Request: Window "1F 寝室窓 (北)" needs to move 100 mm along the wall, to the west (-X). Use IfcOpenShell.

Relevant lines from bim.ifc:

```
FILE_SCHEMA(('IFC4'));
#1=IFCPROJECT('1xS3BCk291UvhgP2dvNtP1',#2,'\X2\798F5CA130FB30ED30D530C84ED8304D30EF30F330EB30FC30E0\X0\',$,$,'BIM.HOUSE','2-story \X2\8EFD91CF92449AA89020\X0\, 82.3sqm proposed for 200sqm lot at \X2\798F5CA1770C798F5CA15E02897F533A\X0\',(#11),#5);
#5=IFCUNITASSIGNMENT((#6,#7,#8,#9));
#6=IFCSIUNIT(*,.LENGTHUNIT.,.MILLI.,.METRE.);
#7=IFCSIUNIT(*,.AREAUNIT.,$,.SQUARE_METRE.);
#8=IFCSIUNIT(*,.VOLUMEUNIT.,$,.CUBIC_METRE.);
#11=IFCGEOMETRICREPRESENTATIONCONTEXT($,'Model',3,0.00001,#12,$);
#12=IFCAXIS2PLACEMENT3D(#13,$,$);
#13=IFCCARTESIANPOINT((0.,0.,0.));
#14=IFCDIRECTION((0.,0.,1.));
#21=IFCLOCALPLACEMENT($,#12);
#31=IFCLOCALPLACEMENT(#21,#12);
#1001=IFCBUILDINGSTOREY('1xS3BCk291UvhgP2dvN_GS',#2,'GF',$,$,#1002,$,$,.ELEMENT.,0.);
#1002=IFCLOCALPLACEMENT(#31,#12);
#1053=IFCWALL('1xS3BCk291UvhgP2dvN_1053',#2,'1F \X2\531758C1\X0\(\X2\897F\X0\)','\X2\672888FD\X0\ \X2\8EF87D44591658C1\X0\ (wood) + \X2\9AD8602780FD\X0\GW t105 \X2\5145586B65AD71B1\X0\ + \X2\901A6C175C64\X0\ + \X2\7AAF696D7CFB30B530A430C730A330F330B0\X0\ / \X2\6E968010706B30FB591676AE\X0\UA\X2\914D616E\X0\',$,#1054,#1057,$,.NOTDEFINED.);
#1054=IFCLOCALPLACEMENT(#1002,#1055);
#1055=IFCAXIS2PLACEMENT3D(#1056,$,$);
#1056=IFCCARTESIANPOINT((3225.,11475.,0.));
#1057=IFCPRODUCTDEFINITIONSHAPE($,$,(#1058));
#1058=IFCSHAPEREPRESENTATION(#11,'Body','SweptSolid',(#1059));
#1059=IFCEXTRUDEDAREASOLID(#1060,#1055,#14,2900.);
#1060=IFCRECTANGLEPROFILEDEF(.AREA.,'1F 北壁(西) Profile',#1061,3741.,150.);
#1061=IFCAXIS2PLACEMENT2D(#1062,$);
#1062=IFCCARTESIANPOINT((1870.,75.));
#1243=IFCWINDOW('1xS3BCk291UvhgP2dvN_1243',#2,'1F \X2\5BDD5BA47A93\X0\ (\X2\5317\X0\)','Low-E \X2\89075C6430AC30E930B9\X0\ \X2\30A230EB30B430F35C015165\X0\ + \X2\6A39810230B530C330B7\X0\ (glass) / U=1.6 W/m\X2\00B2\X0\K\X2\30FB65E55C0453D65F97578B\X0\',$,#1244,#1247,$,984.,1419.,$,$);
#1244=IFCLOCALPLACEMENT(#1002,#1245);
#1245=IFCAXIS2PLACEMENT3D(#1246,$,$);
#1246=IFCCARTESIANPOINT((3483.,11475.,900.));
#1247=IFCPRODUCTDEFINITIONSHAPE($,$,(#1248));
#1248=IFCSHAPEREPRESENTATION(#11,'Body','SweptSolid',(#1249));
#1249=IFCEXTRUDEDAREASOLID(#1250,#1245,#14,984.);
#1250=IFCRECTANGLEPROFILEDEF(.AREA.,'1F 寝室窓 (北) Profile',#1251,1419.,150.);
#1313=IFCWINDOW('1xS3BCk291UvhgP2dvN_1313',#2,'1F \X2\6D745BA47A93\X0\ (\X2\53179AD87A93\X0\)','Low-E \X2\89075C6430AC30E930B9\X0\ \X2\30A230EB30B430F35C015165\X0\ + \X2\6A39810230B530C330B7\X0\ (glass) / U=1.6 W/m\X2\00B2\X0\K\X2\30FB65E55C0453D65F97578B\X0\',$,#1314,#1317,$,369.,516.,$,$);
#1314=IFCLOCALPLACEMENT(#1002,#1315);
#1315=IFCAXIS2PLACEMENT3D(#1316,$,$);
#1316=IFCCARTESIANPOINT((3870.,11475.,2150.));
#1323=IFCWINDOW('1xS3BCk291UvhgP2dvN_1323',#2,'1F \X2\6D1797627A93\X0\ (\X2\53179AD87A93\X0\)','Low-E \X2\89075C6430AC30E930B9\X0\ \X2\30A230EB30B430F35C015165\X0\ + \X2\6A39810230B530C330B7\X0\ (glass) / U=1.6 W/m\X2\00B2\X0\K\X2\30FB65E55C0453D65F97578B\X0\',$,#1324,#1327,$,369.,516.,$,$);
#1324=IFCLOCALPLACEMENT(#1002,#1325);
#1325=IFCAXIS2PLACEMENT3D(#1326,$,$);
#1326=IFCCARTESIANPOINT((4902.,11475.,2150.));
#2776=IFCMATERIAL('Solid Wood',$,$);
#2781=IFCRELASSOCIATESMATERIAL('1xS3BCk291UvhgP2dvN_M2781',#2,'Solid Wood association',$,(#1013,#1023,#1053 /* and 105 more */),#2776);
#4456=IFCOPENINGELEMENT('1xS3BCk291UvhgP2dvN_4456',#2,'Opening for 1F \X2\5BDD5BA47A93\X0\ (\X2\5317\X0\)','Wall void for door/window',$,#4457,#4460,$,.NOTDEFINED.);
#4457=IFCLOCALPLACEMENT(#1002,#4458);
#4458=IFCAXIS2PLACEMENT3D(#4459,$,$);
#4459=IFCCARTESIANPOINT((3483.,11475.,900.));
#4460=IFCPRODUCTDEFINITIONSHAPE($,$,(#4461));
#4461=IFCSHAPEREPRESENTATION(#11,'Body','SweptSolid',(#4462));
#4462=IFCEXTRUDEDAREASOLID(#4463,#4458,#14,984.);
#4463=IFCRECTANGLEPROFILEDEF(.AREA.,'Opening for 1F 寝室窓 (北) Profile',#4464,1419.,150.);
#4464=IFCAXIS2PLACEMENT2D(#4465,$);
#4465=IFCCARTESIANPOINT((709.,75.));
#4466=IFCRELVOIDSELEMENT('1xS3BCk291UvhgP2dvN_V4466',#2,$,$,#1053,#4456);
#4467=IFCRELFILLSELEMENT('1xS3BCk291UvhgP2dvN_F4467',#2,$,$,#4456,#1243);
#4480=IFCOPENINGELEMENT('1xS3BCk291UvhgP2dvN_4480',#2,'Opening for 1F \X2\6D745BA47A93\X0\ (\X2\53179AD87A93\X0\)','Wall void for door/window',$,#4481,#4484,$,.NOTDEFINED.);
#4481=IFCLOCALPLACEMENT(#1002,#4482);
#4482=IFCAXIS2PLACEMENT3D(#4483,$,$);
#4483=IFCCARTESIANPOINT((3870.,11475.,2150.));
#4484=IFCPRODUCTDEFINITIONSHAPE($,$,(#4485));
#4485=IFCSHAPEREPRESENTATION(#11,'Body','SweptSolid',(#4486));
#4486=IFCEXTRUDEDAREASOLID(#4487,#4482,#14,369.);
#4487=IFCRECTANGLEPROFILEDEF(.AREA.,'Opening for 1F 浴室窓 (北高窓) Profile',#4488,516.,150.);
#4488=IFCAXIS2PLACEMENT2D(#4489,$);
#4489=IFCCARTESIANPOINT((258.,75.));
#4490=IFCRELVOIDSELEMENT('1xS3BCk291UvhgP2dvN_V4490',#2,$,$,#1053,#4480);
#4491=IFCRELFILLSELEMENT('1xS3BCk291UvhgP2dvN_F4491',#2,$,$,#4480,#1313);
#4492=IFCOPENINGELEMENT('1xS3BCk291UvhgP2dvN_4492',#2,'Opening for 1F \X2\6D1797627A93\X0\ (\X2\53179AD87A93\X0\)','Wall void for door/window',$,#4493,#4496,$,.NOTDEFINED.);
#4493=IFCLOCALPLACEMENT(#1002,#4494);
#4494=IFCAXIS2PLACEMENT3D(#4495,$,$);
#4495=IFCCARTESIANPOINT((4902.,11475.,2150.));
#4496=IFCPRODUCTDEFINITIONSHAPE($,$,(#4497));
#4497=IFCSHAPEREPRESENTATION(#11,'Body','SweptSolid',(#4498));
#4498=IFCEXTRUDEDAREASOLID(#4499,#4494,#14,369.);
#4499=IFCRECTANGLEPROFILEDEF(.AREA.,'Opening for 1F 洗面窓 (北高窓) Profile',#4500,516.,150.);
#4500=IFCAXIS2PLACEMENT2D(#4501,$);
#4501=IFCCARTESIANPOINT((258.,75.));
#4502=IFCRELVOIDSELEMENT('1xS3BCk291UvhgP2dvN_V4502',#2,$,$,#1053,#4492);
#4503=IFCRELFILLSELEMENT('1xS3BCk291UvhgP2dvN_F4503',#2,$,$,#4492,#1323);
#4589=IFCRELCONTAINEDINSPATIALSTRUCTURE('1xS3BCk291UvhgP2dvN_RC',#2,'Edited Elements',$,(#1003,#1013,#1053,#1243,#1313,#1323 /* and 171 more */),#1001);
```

```python
import ifcopenshell
import ifcopenshell.api.geometry
import ifcopenshell.util.placement
import ifcopenshell.util.unit

model = ifcopenshell.open("bim.ifc")
unit_scale = ifcopenshell.util.unit.calculate_unit_scale(model)

window = model.by_guid("1xS3BCk291UvhgP2dvN_1243")
opening = window.FillsVoids[0].RelatingOpeningElement
wall = opening.VoidsElements[0].RelatingBuildingElement

wall_matrix = ifcopenshell.util.placement.get_local_placement(wall.ObjectPlacement)
shift = wall_matrix[:3, 0] * -0.1 / unit_scale
before = ifcopenshell.util.placement.get_local_placement(window.ObjectPlacement)[:3, 3].copy()

# The window is not placed relative to its opening, so move both.
for product in (opening, window):
    matrix = ifcopenshell.util.placement.get_local_placement(product.ObjectPlacement)
    matrix[:3, 3] += shift
    ifcopenshell.api.geometry.edit_object_placement(model, product=product, matrix=matrix, is_si=False)

after = ifcopenshell.util.placement.get_local_placement(window.ObjectPlacement)[:3, 3]
print("window moved by", (after - before).round(3) + 0.0)

model.write("bim-out.ifc")
```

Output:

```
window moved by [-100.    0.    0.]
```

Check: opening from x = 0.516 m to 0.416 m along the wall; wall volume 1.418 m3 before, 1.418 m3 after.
